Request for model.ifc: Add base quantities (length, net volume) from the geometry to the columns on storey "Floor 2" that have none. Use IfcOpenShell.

First a look at what the model holds.

```python
import ifcopenshell
import ifcopenshell.util.element
import ifcopenshell.util.unit

model = ifcopenshell.open("model.ifc")
print(model.schema)
for unit_type in ("LENGTHUNIT", "AREAUNIT", "VOLUMEUNIT"):
    print(unit_type, ifcopenshell.util.unit.calculate_unit_scale(model, unit_type))
storey = next(s for s in model.by_type("IfcBuildingStorey") if s.Name == "Floor 2")
columns = [e for e in ifcopenshell.util.element.get_decomposition(storey) if e.is_a("IfcColumn")]
for e in sorted(columns, key=lambda e: e.id()):
    print(e.id(), e.is_a(), e.Name, list(ifcopenshell.util.element.get_psets(e, qtos_only=True)), sep=" | ")
```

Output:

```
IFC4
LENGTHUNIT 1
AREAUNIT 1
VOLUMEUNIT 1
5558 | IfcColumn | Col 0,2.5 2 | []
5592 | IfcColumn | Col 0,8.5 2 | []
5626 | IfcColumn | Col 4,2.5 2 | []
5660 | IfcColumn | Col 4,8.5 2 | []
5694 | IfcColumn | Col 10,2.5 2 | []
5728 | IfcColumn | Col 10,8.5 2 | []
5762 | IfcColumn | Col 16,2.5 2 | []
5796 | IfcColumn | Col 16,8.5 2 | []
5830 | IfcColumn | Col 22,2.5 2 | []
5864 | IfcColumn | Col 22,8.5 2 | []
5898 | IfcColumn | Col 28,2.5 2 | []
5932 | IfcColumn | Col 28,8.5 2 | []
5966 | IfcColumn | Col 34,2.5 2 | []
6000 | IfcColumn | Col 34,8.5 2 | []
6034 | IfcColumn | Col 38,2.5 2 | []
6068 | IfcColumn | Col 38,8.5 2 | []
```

```python
import ifcopenshell
import ifcopenshell.api.pset
import ifcopenshell.geom
import ifcopenshell.util.element
import ifcopenshell.util.shape
import ifcopenshell.util.unit

model = ifcopenshell.open("model.ifc")
unit_scale = ifcopenshell.util.unit.calculate_unit_scale(model)
volume_scale = ifcopenshell.util.unit.calculate_unit_scale(model, "VOLUMEUNIT")
settings = ifcopenshell.geom.settings()

storey = next(s for s in model.by_type("IfcBuildingStorey") if s.Name == "Floor 2")
columns = [e for e in ifcopenshell.util.element.get_decomposition(storey) if e.is_a("IfcColumn")]

for e in sorted(columns, key=lambda e: e.id()):
    if ifcopenshell.util.element.get_psets(e, qtos_only=True, should_inherit=False):
        continue
    # Geometry comes back in metres, in the element's own axes.
    shape = ifcopenshell.geom.create_shape(settings, e)
    values = {
        "Length": ifcopenshell.util.shape.get_z(shape.geometry) / unit_scale,
        "NetVolume": ifcopenshell.util.shape.get_volume(shape.geometry) / volume_scale,
    }
    qto = ifcopenshell.api.pset.add_qto(model, product=e, name="Qto_ColumnBaseQuantities")
    ifcopenshell.api.pset.edit_qto(model, qto=qto, properties=values)
    print(e.id(), {k: round(v, 3) for k, v in values.items()})

model.write("model_edited.ifc")
```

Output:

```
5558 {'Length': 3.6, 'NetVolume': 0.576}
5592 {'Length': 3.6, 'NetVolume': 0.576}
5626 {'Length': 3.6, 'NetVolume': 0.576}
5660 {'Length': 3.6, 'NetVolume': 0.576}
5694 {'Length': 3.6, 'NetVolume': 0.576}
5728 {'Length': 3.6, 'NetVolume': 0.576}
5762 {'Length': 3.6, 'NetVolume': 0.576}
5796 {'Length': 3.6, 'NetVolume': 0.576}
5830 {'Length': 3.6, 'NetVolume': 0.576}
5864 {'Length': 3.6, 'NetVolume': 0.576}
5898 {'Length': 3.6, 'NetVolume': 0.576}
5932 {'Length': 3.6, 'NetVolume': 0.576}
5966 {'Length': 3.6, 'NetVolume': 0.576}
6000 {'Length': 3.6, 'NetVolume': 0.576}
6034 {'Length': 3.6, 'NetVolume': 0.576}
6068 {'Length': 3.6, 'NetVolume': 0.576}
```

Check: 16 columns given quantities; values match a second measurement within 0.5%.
